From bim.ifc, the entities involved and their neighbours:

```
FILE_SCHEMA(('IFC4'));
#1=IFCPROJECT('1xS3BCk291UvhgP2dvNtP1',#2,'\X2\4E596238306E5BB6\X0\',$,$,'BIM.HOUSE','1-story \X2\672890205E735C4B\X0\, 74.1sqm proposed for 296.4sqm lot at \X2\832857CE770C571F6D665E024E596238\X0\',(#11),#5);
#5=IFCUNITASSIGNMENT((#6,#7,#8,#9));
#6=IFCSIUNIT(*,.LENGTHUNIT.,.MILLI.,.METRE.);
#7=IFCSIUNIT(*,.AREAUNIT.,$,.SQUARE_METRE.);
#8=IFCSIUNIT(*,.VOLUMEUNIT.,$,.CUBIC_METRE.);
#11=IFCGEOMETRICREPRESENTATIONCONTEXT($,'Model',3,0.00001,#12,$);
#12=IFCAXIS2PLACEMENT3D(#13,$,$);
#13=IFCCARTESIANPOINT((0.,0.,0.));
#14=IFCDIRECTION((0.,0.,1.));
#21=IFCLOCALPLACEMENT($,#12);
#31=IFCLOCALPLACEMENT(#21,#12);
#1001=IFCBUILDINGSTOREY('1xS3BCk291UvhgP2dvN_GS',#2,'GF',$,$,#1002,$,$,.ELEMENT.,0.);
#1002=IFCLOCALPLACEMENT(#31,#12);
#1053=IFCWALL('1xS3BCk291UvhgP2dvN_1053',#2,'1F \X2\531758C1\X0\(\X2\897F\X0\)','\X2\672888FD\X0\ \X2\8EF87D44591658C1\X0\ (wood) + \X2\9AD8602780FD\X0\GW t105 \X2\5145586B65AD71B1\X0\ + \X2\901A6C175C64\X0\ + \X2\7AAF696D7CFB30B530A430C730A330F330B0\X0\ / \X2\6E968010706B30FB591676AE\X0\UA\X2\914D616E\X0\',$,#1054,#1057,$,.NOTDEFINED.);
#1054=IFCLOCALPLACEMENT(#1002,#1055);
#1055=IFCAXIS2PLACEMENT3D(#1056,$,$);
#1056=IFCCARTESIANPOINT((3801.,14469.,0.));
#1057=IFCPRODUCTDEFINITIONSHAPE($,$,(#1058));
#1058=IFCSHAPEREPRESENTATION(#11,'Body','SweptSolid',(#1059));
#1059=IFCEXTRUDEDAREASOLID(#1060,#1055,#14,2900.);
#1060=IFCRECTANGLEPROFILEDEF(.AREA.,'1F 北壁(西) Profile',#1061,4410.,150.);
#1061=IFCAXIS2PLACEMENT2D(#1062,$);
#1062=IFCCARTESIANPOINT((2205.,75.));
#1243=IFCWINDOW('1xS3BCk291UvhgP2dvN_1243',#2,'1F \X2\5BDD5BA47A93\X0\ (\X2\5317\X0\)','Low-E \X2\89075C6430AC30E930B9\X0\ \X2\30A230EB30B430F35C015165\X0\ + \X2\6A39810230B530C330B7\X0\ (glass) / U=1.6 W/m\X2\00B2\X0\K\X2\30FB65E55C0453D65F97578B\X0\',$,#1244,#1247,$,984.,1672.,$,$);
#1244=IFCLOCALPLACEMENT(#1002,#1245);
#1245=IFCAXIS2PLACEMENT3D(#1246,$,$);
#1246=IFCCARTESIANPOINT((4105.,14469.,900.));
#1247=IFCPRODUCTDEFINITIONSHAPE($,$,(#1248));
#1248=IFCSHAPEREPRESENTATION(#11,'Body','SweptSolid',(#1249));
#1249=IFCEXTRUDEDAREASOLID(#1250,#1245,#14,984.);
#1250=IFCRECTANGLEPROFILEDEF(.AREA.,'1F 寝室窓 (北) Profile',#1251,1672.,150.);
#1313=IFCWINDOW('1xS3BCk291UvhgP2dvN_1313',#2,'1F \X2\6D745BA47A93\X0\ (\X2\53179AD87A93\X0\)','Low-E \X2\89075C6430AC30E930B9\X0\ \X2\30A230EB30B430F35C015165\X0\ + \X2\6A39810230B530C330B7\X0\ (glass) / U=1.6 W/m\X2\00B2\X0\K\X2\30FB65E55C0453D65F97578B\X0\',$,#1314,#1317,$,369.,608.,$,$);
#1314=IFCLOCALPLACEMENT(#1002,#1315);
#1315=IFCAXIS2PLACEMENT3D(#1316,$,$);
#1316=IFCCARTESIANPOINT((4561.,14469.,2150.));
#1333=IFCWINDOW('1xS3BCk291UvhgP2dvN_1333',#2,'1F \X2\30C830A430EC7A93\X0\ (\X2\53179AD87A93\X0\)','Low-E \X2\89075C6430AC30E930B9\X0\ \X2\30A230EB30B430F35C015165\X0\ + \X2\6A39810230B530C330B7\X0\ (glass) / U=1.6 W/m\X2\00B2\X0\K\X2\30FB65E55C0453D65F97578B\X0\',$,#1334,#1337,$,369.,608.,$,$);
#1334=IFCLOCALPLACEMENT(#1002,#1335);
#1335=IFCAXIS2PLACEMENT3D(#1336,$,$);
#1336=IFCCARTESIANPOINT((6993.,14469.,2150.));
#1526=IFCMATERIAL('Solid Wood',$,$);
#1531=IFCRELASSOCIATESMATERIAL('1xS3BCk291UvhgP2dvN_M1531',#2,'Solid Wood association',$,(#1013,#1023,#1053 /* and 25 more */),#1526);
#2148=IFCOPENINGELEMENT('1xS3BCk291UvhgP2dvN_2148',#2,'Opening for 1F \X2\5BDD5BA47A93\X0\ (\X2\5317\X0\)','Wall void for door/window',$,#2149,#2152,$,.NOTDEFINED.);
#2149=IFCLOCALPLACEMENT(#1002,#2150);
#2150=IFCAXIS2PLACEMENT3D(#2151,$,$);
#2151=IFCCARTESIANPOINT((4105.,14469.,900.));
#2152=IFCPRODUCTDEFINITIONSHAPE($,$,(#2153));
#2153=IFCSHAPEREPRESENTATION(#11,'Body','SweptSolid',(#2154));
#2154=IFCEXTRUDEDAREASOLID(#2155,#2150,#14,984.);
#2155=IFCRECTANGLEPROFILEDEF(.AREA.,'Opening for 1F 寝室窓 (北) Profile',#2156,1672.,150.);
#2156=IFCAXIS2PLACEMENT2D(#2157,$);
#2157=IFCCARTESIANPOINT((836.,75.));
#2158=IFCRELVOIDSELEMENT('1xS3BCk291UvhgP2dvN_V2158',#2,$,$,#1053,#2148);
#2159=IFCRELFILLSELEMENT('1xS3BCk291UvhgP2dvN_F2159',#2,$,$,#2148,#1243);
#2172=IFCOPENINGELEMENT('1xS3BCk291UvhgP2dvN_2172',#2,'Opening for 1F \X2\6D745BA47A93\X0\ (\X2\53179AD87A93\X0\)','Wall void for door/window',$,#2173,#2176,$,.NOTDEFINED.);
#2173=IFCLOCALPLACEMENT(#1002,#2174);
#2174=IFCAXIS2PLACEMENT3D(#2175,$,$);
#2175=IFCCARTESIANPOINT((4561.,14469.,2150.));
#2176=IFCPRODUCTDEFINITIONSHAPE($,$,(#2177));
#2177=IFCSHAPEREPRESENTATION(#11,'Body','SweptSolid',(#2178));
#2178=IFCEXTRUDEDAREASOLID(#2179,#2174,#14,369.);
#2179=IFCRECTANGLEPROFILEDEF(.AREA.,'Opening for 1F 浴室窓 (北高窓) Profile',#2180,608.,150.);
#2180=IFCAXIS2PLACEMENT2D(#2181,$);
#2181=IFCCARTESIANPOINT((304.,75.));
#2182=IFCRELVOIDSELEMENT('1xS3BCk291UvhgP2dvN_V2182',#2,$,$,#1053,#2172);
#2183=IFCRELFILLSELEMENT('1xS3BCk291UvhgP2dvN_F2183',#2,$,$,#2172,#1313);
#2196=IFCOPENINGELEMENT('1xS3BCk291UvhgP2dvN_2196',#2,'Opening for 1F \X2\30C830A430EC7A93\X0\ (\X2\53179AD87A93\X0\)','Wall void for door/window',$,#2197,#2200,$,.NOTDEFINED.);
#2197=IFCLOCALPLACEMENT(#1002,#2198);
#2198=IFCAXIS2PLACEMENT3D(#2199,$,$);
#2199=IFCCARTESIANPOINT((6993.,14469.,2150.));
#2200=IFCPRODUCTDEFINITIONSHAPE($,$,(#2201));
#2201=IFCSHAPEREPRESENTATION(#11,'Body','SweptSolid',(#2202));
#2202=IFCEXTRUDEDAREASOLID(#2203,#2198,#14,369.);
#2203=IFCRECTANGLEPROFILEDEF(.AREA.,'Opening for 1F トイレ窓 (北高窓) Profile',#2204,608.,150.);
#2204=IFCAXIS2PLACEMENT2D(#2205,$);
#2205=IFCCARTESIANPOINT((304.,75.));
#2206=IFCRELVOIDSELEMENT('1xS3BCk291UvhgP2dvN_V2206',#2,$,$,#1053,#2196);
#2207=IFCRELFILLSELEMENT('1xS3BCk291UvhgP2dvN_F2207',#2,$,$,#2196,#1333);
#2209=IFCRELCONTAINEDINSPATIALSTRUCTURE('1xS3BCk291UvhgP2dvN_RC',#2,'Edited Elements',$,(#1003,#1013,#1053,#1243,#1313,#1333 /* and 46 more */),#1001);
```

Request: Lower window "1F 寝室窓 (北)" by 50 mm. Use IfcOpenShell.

```python
import numpy as np
import ifcopenshell
import ifcopenshell.api.geometry
import ifcopenshell.util.placement
import ifcopenshell.util.unit

model = ifcopenshell.open("bim.ifc")
unit_scale = ifcopenshell.util.unit.calculate_unit_scale(model)

window = model.by_guid("1xS3BCk291UvhgP2dvN_1243")
opening = window.FillsVoids[0].RelatingOpeningElement
dz = -0.05 / unit_scale

shift = np.array([0.0, 0.0, dz])
# The window is not placed relative to its opening, so move both.
for product in (opening, window):
    matrix = ifcopenshell.util.placement.get_local_placement(product.ObjectPlacement)
    matrix[:3, 3] += shift
    ifcopenshell.api.geometry.edit_object_placement(model, product=product, matrix=matrix, is_si=False)

print(f"moved by {dz * unit_scale:+.3f} m")

model.write("bim_edited.ifc")
```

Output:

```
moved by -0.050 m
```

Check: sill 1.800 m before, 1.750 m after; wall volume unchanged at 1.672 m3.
